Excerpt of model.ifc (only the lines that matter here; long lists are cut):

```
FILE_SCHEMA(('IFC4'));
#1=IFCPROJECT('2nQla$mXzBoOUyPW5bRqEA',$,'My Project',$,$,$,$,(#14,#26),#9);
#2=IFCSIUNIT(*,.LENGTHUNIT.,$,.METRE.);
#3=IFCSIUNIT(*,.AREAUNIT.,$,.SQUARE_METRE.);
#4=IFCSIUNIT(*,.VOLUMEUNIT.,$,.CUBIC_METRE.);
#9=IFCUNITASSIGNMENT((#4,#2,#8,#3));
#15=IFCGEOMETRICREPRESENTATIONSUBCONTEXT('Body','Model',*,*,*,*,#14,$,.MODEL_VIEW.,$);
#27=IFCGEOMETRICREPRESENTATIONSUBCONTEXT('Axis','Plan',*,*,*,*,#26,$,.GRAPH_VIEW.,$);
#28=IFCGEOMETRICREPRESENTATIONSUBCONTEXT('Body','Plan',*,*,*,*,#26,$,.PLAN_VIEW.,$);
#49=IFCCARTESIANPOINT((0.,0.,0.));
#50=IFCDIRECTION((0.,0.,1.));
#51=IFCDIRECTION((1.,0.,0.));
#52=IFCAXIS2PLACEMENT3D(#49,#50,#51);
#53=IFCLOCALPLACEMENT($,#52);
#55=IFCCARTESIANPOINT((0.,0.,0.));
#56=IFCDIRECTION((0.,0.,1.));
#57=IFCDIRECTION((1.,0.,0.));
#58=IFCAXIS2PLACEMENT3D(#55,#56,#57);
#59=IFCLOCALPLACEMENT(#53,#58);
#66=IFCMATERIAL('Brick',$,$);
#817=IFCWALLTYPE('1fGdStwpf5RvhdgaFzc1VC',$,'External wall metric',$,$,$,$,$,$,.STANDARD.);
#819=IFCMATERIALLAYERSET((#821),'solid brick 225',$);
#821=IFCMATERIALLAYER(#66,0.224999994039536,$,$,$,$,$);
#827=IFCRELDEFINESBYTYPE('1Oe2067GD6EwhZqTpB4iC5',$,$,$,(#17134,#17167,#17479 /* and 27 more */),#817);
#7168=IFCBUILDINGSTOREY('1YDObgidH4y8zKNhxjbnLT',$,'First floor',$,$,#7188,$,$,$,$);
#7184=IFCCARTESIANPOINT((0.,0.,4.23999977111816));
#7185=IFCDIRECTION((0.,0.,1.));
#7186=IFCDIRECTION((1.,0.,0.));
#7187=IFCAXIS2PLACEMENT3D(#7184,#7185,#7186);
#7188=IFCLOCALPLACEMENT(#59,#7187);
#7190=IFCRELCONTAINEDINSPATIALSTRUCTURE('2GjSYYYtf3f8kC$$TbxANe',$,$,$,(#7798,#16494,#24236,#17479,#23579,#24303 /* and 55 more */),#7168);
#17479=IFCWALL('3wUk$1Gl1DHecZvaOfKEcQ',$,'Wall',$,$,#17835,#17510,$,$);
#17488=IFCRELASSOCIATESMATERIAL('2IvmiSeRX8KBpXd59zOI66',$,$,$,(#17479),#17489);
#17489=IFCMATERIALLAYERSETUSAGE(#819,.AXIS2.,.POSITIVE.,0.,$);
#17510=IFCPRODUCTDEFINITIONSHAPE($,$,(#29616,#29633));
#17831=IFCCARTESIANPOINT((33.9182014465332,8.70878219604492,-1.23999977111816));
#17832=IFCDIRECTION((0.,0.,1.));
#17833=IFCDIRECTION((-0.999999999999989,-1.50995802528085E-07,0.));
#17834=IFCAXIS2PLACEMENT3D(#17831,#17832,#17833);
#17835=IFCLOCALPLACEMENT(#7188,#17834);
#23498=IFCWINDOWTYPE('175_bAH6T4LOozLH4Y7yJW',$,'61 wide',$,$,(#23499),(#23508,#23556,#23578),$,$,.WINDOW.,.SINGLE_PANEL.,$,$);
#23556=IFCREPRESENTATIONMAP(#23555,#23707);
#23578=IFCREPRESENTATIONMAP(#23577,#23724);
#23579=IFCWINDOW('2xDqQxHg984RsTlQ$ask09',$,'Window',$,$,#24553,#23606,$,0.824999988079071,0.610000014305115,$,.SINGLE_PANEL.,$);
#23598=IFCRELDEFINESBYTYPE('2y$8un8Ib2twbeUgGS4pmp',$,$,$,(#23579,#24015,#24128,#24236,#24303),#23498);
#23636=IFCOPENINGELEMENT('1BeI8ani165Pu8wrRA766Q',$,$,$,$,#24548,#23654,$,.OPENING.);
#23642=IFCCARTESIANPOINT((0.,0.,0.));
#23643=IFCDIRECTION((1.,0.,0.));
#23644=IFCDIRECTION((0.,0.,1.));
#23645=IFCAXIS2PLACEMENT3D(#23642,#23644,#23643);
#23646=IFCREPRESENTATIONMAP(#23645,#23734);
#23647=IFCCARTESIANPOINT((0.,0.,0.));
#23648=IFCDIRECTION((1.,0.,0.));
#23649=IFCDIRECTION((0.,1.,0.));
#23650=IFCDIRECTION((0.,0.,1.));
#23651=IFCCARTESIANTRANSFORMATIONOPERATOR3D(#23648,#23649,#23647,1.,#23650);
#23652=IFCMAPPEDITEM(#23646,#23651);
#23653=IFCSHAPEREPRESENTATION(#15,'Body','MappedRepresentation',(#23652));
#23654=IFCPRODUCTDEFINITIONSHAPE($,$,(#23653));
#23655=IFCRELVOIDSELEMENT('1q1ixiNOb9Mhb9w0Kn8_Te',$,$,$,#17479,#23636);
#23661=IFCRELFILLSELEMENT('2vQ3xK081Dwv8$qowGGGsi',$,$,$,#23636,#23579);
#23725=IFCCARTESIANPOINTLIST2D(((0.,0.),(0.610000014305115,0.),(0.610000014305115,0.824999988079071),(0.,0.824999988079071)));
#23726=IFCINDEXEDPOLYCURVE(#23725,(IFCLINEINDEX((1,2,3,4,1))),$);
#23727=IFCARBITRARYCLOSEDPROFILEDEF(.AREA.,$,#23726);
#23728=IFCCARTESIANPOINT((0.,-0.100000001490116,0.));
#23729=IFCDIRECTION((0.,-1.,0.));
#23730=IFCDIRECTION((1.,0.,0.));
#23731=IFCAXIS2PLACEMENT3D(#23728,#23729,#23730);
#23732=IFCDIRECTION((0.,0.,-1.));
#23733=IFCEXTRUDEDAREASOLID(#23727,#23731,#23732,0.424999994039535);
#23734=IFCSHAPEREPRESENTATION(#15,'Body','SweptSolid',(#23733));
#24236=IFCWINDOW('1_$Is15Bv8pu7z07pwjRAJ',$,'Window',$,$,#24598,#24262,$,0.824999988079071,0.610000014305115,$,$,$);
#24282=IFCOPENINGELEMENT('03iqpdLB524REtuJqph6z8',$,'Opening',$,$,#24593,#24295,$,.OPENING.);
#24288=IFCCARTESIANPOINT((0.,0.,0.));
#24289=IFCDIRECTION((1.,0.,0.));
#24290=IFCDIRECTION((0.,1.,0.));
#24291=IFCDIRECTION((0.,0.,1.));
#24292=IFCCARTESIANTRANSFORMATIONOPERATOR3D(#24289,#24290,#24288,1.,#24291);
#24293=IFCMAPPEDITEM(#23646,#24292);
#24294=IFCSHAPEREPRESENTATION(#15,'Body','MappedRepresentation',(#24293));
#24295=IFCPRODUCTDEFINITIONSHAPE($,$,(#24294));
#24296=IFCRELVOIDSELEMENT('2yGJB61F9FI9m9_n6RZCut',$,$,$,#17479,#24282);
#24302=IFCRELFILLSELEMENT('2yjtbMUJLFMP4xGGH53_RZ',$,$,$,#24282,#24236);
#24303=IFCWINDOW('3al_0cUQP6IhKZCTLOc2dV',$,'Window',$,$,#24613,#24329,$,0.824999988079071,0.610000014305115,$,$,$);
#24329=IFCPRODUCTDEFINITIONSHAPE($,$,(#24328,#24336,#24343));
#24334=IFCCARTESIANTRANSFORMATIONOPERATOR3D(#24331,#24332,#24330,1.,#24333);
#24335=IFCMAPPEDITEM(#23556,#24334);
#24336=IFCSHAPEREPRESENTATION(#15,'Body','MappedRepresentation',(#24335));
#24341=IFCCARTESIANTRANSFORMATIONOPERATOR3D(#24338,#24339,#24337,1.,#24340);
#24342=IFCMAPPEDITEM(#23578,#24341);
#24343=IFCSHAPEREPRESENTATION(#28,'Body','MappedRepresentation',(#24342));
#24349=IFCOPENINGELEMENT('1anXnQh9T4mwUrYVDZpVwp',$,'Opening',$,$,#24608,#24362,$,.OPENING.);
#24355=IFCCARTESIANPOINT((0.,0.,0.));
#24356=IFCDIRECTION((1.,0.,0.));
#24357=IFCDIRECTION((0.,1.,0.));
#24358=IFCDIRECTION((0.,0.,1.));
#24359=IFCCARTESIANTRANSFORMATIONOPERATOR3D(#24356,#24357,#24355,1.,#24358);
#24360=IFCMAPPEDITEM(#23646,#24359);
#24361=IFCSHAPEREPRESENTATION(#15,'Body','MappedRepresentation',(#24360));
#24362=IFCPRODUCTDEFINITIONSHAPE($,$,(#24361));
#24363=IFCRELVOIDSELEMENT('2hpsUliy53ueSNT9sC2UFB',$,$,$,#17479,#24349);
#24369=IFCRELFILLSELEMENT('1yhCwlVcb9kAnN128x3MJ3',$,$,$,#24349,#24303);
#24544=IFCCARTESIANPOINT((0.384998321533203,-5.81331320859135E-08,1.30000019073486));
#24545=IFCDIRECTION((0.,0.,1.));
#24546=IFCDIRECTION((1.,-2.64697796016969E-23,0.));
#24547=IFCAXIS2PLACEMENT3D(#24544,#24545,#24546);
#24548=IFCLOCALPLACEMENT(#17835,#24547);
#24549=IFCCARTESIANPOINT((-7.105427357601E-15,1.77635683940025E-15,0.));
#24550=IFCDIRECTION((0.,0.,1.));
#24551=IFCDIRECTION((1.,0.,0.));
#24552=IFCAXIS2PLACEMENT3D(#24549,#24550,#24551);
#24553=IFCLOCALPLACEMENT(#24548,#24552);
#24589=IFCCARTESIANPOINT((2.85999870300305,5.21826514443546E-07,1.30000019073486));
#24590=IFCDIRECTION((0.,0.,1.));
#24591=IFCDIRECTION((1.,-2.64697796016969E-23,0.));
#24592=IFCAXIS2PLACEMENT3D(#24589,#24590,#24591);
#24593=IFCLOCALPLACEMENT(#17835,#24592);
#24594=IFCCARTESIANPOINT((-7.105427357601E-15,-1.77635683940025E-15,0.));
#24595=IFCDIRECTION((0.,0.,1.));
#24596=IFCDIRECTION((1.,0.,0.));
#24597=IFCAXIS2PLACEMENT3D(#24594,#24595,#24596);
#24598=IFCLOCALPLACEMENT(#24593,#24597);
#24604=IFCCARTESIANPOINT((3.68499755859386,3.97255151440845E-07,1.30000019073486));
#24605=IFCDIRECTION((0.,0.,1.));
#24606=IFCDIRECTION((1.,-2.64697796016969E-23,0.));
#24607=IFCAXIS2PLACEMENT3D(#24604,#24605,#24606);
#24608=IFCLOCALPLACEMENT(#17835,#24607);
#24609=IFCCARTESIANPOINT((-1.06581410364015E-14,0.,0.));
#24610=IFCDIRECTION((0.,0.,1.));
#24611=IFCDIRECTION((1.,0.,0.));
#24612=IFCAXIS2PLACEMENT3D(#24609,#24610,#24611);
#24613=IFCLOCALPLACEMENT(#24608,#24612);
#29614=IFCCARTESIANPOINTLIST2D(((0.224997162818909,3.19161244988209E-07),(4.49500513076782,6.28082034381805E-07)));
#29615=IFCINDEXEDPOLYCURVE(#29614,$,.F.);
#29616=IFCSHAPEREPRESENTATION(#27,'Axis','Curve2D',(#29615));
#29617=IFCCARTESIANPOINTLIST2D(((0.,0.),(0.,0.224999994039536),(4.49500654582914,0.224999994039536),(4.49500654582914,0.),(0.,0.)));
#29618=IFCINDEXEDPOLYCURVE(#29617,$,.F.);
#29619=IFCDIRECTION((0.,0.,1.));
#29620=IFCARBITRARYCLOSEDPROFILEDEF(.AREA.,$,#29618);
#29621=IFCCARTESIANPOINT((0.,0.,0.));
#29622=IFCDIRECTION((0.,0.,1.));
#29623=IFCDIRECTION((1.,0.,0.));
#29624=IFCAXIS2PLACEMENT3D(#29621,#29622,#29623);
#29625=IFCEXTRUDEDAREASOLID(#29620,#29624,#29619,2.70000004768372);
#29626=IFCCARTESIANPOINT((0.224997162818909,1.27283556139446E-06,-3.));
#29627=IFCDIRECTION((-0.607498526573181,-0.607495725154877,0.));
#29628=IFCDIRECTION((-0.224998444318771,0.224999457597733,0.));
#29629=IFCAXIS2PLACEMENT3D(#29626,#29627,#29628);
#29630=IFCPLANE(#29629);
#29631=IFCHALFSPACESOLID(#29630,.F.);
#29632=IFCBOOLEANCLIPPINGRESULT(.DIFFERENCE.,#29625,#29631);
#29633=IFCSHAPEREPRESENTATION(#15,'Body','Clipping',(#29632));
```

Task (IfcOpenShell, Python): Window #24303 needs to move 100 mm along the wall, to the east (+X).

```python
import ifcopenshell
import ifcopenshell.api.geometry
import ifcopenshell.util.placement

model = ifcopenshell.open("model.ifc")

window = model.by_guid("3al_0cUQP6IhKZCTLOc2dV")
opening = window.FillsVoids[0].RelatingOpeningElement
wall = opening.VoidsElements[0].RelatingBuildingElement

wall_matrix = ifcopenshell.util.placement.get_local_placement(wall.ObjectPlacement)
shift = wall_matrix[:3, 0] * -0.1
before = ifcopenshell.util.placement.get_local_placement(window.ObjectPlacement)[:3, 3].copy()

# The window is placed relative to its opening, so it follows when the opening moves.
matrix = ifcopenshell.util.placement.get_local_placement(opening.ObjectPlacement)
matrix[:3, 3] += shift
ifcopenshell.api.geometry.edit_object_placement(
    model, product=opening, matrix=matrix, is_si=False, should_transform_children=True
)

after = ifcopenshell.util.placement.get_local_placement(window.ObjectPlacement)[:3, 3]
print("window moved by", (after - before).round(3) + 0.0)

model.write("model_edited.ifc")
```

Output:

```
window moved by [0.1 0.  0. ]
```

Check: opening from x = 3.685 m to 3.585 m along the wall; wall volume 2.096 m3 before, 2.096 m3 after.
